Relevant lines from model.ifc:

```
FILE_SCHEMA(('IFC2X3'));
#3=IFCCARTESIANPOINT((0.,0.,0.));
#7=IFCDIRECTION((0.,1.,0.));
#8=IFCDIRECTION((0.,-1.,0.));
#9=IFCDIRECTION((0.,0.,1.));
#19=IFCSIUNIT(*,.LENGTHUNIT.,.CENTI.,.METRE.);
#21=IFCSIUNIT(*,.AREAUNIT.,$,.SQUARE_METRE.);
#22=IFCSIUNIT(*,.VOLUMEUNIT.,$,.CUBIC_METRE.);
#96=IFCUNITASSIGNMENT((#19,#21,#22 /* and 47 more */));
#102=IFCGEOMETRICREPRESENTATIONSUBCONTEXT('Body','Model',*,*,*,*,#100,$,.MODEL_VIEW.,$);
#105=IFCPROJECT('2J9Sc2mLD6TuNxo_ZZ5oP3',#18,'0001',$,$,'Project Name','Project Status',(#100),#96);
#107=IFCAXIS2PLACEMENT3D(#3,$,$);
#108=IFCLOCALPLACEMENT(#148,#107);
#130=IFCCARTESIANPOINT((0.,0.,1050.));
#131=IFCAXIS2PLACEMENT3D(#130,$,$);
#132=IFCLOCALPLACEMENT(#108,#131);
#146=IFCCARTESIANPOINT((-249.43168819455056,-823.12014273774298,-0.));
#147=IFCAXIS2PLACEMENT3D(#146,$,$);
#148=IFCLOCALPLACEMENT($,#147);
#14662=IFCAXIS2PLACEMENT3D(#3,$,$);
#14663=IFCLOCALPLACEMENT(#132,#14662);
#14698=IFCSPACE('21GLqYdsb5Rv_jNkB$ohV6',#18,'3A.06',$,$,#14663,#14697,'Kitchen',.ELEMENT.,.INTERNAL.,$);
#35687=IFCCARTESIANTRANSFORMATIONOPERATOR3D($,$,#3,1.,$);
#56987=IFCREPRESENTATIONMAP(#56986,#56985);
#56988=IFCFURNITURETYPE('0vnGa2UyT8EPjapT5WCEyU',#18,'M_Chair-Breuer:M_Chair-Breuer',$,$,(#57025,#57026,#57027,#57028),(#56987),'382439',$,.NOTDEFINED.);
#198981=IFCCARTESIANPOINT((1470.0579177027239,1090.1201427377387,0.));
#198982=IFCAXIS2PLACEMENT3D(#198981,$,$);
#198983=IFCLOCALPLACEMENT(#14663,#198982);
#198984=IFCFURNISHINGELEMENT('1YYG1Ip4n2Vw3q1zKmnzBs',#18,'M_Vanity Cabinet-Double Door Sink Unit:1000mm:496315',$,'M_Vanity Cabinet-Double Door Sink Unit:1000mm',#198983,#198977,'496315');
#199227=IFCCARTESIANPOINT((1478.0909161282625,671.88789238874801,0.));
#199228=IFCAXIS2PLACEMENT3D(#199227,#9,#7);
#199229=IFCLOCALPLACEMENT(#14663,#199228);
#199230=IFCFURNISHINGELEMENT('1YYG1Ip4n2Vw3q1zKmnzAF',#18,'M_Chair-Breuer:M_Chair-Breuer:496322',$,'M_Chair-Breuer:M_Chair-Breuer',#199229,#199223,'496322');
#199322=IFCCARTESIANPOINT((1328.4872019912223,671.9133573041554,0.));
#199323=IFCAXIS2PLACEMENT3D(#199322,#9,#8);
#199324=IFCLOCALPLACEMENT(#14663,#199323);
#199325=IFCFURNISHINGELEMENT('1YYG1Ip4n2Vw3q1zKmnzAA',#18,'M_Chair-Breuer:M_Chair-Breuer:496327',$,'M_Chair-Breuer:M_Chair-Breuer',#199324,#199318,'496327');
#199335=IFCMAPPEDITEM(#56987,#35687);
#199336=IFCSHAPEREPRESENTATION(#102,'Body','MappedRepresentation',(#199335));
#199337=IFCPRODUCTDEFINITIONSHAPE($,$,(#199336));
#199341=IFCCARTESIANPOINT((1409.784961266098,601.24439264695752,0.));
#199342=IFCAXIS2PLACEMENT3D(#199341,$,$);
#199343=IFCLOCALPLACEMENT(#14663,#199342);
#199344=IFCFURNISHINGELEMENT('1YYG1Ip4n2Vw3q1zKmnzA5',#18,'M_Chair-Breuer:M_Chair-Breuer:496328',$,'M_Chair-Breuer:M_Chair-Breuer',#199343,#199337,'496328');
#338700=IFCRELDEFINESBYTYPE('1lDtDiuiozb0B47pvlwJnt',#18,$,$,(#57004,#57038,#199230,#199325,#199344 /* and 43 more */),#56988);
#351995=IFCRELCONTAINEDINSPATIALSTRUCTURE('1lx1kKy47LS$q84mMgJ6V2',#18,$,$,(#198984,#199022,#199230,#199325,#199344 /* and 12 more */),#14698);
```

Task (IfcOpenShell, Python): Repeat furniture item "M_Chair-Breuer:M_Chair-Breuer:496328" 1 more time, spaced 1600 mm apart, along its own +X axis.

```python
import ifcopenshell
import ifcopenshell.api.geometry
import ifcopenshell.api.root
import ifcopenshell.util.element
import ifcopenshell.util.placement
import ifcopenshell.util.unit

model = ifcopenshell.open("model.ifc")
unit_scale = ifcopenshell.util.unit.calculate_unit_scale(model)


def reuse_history(source, copy):
    """copy_class also copies each property set's owner history, people and application; keep the originals."""
    for rel in copy.IsDefinedBy:
        if rel.is_a("IfcRelDefinesByProperties") and (history := rel.RelatingPropertyDefinition.OwnerHistory):
            rel.RelatingPropertyDefinition.OwnerHistory = source.OwnerHistory
            ifcopenshell.util.element.remove_deep2(model, history)


source = model.by_guid("1YYG1Ip4n2Vw3q1zKmnzA5")
base = ifcopenshell.util.placement.get_local_placement(source.ObjectPlacement)
step = base[:3, 0] * 1.6 / unit_scale

for i in range(1, 2):
    copy = ifcopenshell.api.root.copy_class(model, product=source)
    copy.Representation = ifcopenshell.util.element.copy_deep(
        model, source.Representation, exclude=["IfcGeometricRepresentationContext", "IfcRepresentationMap"]
    )
    copy.Name = "M_Chair-Breuer:M_Chair-Breuer"
    copy.Tag = None
    reuse_history(source, copy)
    matrix = base.copy()
    matrix[:3, 3] += i * step
    print("added at", matrix[:3, 3].round(3) + 0.0)
    ifcopenshell.api.geometry.edit_object_placement(model, product=copy, matrix=matrix, is_si=False)

model.write("model-out.ifc")
```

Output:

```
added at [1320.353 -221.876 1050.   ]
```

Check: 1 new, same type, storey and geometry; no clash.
